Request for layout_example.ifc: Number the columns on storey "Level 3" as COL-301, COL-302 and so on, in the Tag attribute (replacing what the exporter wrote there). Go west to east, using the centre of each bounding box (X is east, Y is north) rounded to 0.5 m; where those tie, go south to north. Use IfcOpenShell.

First a look at what the model holds.

```python
import ifcopenshell
import ifcopenshell.util.element
import ifcopenshell.util.placement

model = ifcopenshell.open("layout_example.ifc")
print(model.schema)
storey = next(s for s in model.by_type("IfcBuildingStorey") if s.Name == "Level 3")
columns = [e for e in ifcopenshell.util.element.get_decomposition(storey) if e.is_a("IfcColumn")]
for e in sorted(columns, key=lambda e: e.id()):
    origin = ifcopenshell.util.placement.get_local_placement(e.ObjectPlacement)[:3, 3]
    print(e.id(), e.Tag, e.Name, origin.round(2) + 0.0, sep=" | ")
```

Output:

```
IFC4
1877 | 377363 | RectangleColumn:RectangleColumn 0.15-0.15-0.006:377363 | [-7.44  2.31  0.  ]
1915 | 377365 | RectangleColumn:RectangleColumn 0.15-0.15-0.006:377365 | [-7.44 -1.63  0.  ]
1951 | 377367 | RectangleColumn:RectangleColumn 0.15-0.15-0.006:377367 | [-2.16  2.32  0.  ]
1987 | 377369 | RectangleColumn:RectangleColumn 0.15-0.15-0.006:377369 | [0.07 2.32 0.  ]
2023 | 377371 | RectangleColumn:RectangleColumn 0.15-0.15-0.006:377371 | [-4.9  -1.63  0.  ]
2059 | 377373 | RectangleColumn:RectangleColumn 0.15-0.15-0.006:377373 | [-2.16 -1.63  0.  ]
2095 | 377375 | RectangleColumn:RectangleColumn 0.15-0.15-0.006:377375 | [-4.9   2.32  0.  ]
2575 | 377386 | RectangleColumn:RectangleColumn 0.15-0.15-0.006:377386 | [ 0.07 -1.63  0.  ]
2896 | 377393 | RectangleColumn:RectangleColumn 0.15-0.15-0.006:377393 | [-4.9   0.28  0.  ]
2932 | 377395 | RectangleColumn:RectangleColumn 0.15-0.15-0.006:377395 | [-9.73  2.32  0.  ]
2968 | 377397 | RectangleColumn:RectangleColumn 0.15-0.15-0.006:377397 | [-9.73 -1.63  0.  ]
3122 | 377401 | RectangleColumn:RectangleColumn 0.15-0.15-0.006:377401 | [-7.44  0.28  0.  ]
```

```python
import ifcopenshell
import ifcopenshell.geom
import ifcopenshell.util.element
import ifcopenshell.util.shape

model = ifcopenshell.open("layout_example.ifc")
settings = ifcopenshell.geom.settings()
settings.set("use-world-coords", True)


def centre(element):
    shape = ifcopenshell.geom.create_shape(settings, element)
    return ifcopenshell.util.shape.get_bbox_centroid(shape.geometry)


storey = next(s for s in model.by_type("IfcBuildingStorey") if s.Name == "Level 3")
columns = [e for e in ifcopenshell.util.element.get_decomposition(storey) if e.is_a("IfcColumn")]

# Insertion points can sit at a corner or the storey origin, so sort by the geometry (in metres).
centres = {e: centre(e) for e in columns}
columns.sort(key=lambda e: (round(centres[e][0] / 0.5), centres[e][1]))

for i, e in enumerate(columns, start=1):
    number = f"COL-3{i:02d}"
    e.Tag = number
    print(e.id(), number)

model.write("layout_example_updated.ifc")
```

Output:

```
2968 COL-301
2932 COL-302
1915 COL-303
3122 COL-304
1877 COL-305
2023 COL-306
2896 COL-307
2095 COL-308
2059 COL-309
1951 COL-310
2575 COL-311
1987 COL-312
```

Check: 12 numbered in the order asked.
